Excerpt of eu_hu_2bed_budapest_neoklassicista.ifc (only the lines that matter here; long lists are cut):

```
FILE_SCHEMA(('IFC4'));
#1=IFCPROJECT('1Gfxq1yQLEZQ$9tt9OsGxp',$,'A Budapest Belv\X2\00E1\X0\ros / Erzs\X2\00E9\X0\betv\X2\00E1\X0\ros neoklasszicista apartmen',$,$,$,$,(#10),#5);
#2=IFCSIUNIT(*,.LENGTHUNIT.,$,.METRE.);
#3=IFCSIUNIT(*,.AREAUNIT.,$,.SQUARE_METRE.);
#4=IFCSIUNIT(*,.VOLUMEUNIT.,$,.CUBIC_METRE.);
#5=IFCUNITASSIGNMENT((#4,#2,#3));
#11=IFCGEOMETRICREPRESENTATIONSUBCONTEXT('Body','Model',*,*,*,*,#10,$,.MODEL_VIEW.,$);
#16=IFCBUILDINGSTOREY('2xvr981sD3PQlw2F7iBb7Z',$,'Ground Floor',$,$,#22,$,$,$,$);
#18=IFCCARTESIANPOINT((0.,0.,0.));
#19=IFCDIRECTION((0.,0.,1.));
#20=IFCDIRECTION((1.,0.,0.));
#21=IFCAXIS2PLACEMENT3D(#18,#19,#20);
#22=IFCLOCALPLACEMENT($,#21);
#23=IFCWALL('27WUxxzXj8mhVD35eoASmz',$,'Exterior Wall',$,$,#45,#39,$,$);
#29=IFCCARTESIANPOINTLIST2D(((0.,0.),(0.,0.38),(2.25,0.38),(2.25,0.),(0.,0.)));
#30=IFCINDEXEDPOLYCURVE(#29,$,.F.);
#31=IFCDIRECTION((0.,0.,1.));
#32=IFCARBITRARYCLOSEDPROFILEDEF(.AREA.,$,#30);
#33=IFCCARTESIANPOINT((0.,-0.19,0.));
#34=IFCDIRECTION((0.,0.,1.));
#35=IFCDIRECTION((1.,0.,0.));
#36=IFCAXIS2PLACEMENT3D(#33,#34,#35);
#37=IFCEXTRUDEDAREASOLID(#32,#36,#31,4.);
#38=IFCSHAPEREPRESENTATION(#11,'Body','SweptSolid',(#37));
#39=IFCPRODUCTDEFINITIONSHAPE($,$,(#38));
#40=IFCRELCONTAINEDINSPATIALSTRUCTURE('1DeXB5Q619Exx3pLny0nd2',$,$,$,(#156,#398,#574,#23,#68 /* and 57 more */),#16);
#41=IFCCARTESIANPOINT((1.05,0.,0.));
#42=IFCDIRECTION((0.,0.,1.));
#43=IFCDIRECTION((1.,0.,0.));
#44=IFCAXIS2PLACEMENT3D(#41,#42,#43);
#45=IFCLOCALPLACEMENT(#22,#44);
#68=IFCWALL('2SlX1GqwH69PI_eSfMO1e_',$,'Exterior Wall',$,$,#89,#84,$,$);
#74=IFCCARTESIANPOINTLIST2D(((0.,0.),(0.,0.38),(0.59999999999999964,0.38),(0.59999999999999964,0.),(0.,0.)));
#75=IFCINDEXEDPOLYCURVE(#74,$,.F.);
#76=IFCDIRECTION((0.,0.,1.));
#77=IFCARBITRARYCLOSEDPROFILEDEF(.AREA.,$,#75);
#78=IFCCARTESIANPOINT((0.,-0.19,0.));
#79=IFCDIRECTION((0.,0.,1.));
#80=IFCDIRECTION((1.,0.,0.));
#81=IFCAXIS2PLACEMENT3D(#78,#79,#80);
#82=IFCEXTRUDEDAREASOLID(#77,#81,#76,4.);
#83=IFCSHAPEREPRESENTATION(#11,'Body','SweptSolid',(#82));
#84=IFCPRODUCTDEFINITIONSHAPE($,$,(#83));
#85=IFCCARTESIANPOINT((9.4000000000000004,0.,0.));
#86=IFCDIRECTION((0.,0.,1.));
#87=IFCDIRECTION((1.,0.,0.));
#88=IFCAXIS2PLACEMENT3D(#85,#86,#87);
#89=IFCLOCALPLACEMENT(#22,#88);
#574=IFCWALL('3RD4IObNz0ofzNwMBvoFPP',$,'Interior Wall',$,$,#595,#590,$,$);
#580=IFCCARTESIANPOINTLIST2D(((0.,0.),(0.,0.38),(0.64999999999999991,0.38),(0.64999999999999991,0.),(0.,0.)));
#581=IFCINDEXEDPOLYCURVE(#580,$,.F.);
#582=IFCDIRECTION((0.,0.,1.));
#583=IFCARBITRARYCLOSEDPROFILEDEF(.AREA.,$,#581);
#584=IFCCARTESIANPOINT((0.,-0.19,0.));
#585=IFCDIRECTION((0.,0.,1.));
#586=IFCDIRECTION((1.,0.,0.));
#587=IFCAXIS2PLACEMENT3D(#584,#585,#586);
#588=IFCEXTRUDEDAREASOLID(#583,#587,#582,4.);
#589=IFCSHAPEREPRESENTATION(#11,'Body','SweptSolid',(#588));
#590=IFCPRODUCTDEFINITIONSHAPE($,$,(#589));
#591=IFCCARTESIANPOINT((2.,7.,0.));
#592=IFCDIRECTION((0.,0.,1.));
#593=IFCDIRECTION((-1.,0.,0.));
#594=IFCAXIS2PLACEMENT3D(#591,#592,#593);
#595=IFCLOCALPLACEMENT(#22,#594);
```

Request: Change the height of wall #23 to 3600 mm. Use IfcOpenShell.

```python
import ifcopenshell
import ifcopenshell.geom
import ifcopenshell.util.representation
import ifcopenshell.util.shape
import ifcopenshell.util.unit

model = ifcopenshell.open("eu_hu_2bed_budapest_neoklassicista.ifc")
unit_scale = ifcopenshell.util.unit.calculate_unit_scale(model)
settings = ifcopenshell.geom.settings()


def volume(element):
    """Net volume in cubic metres, openings subtracted."""
    shape = ifcopenshell.geom.create_shape(settings, element)
    return ifcopenshell.util.shape.get_volume(shape.geometry)


wall = model.by_guid("27WUxxzXj8mhVD35eoASmz")
before = volume(wall)

body = ifcopenshell.util.representation.get_representation(wall, "Model", "Body")
solid = body.Items[0]
old_height = solid.Depth
solid.Depth = 3.6 / unit_scale
after = volume(wall)

print(f"height {old_height:g} -> {solid.Depth:g}, volume {before:.3f} -> {after:.3f} m3")

model.write("eu_hu_2bed_budapest_neoklassicista_rev.ifc")
```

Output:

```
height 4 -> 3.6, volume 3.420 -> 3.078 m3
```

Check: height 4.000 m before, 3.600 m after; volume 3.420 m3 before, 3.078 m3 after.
